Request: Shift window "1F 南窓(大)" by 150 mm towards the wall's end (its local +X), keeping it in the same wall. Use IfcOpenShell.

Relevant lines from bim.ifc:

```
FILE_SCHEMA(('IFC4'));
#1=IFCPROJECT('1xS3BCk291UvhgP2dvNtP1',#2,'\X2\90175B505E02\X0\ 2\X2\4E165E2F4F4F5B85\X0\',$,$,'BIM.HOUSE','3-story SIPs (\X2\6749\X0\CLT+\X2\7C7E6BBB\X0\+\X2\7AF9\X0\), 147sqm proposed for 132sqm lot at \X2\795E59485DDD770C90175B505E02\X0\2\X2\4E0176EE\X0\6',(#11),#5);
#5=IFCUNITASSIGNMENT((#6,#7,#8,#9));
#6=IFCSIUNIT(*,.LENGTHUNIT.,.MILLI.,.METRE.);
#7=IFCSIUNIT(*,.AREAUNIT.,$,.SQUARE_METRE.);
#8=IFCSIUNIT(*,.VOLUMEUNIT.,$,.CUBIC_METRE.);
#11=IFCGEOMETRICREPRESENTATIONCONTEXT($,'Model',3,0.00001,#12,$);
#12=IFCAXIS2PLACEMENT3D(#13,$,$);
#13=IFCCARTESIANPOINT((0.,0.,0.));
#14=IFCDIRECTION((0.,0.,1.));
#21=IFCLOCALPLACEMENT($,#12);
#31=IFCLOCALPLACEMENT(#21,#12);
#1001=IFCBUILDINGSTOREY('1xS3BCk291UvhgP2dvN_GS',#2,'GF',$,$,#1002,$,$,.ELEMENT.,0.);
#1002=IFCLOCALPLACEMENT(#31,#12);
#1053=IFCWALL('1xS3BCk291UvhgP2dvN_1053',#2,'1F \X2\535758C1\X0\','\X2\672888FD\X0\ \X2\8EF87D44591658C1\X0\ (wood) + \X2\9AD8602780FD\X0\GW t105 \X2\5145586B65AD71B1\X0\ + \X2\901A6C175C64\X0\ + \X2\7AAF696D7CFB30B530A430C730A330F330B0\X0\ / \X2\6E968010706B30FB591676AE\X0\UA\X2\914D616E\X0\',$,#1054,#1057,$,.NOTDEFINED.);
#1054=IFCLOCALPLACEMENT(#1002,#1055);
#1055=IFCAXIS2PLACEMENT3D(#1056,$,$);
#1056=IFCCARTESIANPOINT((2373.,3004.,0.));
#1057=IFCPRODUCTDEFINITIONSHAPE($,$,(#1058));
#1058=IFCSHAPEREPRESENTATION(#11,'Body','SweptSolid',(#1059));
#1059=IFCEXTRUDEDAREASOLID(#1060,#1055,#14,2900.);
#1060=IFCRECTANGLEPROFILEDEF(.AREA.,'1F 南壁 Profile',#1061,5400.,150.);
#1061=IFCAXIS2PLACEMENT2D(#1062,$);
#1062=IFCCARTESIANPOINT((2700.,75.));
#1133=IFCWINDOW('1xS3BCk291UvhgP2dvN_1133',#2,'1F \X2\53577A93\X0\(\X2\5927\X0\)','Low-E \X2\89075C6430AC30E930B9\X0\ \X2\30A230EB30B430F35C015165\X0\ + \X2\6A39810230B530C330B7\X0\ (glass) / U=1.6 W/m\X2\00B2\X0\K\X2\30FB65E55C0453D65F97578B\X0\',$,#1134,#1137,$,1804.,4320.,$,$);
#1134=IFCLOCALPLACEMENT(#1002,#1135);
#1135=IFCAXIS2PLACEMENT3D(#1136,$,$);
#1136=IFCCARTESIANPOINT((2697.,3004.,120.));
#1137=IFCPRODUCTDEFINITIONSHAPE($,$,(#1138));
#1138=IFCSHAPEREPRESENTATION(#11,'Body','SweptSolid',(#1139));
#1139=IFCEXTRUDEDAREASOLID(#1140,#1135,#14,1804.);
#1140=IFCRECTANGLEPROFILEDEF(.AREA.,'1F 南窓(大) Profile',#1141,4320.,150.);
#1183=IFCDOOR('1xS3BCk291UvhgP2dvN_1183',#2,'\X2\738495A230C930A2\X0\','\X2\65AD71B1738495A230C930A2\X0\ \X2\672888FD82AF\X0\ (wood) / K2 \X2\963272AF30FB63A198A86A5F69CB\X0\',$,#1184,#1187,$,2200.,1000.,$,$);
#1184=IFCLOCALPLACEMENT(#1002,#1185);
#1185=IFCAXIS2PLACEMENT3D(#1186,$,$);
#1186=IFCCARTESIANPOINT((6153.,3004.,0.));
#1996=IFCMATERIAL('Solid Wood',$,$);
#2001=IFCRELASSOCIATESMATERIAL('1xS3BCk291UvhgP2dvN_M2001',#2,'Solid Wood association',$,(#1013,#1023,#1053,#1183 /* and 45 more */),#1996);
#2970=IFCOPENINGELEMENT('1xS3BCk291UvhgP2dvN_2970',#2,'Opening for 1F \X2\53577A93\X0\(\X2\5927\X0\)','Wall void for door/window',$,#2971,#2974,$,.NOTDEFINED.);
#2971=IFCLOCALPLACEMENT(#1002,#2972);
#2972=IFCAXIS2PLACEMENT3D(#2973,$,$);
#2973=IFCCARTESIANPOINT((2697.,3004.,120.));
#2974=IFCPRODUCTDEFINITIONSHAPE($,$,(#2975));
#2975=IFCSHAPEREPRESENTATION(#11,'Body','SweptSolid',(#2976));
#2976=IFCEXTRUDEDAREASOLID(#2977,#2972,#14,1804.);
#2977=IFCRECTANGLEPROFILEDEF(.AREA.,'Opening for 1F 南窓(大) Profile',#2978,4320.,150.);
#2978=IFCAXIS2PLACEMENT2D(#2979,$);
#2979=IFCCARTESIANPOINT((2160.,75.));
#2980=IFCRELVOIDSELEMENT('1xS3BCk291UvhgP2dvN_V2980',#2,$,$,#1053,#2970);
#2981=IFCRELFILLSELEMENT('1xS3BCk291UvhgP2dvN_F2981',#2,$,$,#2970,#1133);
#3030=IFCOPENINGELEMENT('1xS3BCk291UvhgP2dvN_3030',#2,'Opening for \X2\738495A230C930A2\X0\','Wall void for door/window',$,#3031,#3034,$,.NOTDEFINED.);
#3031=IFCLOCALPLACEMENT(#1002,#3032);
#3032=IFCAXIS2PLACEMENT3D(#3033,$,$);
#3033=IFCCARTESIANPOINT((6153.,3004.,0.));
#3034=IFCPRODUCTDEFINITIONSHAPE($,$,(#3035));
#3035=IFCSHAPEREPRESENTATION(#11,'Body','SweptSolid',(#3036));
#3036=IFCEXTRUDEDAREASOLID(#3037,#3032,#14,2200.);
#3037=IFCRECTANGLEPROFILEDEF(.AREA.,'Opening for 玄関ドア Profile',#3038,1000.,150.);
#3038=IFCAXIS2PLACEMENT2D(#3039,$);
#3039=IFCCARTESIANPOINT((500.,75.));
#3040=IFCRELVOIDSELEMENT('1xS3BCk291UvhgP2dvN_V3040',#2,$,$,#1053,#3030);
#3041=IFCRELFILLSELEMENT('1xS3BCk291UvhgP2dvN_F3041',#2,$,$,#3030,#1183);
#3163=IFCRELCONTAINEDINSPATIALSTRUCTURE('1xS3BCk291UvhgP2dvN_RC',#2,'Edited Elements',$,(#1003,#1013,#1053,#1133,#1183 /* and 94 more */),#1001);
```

```python
import ifcopenshell
import ifcopenshell.api.geometry
import ifcopenshell.util.placement
import ifcopenshell.util.unit

model = ifcopenshell.open("bim.ifc")
unit_scale = ifcopenshell.util.unit.calculate_unit_scale(model)

window = model.by_guid("1xS3BCk291UvhgP2dvN_1133")
opening = window.FillsVoids[0].RelatingOpeningElement
wall = opening.VoidsElements[0].RelatingBuildingElement

wall_matrix = ifcopenshell.util.placement.get_local_placement(wall.ObjectPlacement)
shift = wall_matrix[:3, 0] * 0.15 / unit_scale
before = ifcopenshell.util.placement.get_local_placement(window.ObjectPlacement)[:3, 3].copy()

# The window is not placed relative to its opening, so move both.
for product in (opening, window):
    matrix = ifcopenshell.util.placement.get_local_placement(product.ObjectPlacement)
    matrix[:3, 3] += shift
    ifcopenshell.api.geometry.edit_object_placement(model, product=product, matrix=matrix, is_si=False)

after = ifcopenshell.util.placement.get_local_placement(window.ObjectPlacement)[:3, 3]
print("window moved by", (after - before).round(3) + 0.0)

model.write("bim_rev.ifc")
```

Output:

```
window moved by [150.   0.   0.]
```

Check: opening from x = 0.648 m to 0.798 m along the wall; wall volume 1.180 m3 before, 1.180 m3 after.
